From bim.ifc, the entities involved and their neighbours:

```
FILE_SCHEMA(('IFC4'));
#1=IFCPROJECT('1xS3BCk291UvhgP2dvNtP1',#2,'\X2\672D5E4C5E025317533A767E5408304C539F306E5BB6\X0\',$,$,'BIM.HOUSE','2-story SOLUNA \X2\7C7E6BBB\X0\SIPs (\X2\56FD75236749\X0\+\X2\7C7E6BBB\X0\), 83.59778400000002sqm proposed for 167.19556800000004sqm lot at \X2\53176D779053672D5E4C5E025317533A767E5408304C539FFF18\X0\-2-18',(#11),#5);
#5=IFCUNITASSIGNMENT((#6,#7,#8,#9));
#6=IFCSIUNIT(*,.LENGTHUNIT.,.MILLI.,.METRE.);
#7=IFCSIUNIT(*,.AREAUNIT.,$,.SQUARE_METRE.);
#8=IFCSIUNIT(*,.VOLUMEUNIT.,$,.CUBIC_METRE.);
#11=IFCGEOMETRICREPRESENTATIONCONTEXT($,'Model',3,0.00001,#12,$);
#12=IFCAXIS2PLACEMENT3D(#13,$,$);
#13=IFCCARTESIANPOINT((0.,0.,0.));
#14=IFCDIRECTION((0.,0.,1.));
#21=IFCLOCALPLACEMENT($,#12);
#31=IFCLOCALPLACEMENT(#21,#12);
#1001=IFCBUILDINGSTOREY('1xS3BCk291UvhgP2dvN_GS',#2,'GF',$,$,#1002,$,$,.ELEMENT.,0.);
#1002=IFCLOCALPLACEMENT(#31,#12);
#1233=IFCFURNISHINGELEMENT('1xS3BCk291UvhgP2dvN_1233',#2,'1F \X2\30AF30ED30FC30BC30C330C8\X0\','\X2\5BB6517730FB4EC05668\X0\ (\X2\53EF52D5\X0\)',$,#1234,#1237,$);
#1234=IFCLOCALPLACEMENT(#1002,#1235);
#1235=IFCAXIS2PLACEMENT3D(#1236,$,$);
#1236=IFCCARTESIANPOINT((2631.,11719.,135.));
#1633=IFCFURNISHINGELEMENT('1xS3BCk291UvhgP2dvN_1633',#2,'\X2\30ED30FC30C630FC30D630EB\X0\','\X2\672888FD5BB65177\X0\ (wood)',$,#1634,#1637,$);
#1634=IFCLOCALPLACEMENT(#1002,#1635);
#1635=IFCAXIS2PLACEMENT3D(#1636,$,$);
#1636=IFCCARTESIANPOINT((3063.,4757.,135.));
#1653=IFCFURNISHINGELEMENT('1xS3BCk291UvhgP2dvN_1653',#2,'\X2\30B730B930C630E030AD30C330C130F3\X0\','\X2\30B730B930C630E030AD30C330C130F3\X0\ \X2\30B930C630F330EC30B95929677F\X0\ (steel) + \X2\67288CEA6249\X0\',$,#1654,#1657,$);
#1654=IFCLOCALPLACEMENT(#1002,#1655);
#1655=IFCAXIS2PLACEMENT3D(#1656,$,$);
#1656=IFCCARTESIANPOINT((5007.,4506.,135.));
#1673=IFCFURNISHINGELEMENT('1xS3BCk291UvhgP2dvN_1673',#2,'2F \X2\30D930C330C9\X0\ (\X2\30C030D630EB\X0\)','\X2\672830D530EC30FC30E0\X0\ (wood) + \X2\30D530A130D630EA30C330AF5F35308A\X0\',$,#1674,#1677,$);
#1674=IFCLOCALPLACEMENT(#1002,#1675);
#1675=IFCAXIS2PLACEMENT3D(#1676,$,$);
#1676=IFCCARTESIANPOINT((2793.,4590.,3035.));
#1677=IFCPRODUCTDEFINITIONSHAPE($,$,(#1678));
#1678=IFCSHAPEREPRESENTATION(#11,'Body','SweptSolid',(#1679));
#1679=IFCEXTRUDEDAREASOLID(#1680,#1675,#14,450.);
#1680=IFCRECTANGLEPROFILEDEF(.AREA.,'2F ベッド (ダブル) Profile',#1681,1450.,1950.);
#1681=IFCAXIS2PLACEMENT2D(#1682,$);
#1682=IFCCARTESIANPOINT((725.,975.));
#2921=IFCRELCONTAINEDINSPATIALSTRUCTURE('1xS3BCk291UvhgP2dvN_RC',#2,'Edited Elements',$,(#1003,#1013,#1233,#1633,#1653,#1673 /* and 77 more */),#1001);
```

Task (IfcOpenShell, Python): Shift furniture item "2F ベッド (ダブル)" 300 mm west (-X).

```python
import ifcopenshell
import ifcopenshell.api.geometry
import ifcopenshell.util.placement

model = ifcopenshell.open("bim.ifc")

item = model.by_id(1673)
matrix = ifcopenshell.util.placement.get_local_placement(item.ObjectPlacement)
matrix[0, 3] -= 300.0
ifcopenshell.api.geometry.edit_object_placement(model, product=item, matrix=matrix, is_si=False)

print(ifcopenshell.util.placement.get_local_placement(item.ObjectPlacement).round(3) + 0.0)

model.write("bim_v2.ifc")
```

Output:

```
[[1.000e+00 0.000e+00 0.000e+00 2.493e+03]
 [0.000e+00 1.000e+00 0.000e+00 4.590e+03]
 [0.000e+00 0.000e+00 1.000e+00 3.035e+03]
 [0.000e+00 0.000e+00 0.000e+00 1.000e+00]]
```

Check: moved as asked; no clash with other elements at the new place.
